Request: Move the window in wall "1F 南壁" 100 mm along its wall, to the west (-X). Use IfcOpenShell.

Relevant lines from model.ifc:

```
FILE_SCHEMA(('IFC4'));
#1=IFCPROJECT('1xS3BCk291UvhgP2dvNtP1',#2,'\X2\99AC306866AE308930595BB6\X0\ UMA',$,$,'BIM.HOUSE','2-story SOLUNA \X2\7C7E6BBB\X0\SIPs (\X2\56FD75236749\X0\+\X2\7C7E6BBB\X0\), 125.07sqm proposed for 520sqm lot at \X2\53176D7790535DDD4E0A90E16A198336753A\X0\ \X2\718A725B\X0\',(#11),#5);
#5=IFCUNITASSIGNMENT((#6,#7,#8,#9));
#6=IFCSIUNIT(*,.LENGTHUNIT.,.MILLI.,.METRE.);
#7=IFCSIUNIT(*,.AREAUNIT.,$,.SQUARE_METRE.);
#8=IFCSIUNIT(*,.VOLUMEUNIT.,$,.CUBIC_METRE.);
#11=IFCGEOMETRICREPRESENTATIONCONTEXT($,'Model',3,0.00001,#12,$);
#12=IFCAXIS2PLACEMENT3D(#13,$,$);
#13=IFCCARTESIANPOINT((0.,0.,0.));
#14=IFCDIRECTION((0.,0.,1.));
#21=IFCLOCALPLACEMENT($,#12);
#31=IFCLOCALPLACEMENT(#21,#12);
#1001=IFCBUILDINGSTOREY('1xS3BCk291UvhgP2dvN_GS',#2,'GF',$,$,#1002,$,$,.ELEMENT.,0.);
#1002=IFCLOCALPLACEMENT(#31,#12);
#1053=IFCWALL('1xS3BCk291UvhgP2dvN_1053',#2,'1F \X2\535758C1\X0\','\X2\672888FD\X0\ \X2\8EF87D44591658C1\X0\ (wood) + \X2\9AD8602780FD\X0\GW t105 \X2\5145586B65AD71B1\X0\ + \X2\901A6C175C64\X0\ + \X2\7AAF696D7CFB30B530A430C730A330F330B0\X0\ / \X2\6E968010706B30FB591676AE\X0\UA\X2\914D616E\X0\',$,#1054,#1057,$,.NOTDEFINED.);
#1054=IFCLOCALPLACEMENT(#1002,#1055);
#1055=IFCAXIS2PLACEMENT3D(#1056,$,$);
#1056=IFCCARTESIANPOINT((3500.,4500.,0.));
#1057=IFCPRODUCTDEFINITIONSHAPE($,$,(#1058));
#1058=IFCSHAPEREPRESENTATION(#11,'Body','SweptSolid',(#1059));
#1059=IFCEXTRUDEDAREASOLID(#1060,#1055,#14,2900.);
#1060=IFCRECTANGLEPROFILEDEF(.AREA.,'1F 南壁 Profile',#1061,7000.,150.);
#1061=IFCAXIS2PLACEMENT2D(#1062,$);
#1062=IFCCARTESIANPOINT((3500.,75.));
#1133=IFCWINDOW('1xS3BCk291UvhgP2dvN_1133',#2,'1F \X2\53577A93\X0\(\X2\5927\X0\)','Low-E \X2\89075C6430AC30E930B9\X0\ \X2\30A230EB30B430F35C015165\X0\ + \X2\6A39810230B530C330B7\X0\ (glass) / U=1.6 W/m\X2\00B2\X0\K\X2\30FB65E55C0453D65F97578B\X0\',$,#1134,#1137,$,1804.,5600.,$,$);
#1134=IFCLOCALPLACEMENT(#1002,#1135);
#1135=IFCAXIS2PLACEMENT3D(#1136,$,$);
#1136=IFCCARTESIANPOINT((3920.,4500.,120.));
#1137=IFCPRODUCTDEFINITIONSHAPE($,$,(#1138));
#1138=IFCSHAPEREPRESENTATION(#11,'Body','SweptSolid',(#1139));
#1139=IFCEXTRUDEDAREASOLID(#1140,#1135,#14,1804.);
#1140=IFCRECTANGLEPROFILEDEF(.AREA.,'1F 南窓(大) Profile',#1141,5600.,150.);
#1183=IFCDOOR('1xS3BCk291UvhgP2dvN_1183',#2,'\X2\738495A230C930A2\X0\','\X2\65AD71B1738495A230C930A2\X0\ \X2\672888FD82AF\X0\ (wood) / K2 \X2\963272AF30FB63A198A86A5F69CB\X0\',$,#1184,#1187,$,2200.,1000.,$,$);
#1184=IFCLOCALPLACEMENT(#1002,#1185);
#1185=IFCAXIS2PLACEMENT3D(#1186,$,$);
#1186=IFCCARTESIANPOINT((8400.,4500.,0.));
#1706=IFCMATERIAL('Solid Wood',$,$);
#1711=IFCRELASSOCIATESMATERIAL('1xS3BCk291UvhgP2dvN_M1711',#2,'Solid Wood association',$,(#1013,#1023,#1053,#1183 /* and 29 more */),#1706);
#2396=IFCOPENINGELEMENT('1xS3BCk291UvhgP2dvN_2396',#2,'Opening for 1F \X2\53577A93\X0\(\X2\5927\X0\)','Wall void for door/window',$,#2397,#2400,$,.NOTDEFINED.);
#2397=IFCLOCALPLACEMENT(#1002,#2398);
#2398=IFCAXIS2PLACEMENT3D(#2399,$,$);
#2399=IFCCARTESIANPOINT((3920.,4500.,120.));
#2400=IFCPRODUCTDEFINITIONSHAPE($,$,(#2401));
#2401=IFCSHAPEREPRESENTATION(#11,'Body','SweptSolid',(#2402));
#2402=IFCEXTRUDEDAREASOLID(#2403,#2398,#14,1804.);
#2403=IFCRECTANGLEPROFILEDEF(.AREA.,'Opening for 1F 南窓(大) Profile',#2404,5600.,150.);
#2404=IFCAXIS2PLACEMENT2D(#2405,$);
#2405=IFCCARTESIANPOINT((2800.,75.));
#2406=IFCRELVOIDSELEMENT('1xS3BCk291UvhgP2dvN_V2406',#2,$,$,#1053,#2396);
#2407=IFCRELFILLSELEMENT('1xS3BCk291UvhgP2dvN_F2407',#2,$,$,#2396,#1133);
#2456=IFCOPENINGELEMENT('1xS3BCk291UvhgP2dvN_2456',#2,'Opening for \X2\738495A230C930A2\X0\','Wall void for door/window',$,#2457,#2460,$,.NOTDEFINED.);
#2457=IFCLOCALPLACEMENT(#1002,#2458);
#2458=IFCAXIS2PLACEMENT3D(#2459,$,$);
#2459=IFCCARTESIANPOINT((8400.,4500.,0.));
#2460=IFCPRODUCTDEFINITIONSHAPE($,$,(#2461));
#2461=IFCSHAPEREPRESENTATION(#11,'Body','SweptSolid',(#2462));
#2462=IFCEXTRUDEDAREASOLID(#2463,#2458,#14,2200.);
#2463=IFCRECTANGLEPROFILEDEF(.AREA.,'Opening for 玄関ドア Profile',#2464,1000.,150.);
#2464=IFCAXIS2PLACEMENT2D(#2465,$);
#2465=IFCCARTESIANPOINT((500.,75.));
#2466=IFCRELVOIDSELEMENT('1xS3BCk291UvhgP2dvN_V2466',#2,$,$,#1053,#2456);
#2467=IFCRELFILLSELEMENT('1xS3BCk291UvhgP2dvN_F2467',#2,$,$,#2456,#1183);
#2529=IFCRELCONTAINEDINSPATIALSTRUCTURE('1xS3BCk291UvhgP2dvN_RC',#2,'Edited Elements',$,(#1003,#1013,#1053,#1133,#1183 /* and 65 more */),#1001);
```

```python
import ifcopenshell
import ifcopenshell.api.geometry
import ifcopenshell.util.placement

model = ifcopenshell.open("model.ifc")

window = model.by_guid("1xS3BCk291UvhgP2dvN_1133")
opening = window.FillsVoids[0].RelatingOpeningElement
wall = opening.VoidsElements[0].RelatingBuildingElement

wall_matrix = ifcopenshell.util.placement.get_local_placement(wall.ObjectPlacement)
shift = wall_matrix[:3, 0] * -100.0
before = ifcopenshell.util.placement.get_local_placement(window.ObjectPlacement)[:3, 3].copy()

# The window is not placed relative to its opening, so move both.
for product in (opening, window):
    matrix = ifcopenshell.util.placement.get_local_placement(product.ObjectPlacement)
    matrix[:3, 3] += shift
    ifcopenshell.api.geometry.edit_object_placement(model, product=product, matrix=matrix, is_si=False)

after = ifcopenshell.util.placement.get_local_placement(window.ObjectPlacement)[:3, 3]
print("window moved by", (after - before).round(3) + 0.0)

model.write("model_updated.ifc")
```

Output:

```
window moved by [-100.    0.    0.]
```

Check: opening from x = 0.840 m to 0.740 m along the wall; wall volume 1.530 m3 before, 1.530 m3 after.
